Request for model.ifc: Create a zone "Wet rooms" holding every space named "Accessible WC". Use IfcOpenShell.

First a look at what the model holds.

```python
import ifcopenshell

model = ifcopenshell.open("model.ifc")
print(model.schema)
seen = {}
for space in model.by_type("IfcSpace"):
    seen[space.LongName] = seen.get(space.LongName, 0) + 1
for name, count in sorted(seen.items(), key=str):
    print(count, "x", name)
print("zones:", [z.Name for z in model.by_type("IfcZone")][:20])
```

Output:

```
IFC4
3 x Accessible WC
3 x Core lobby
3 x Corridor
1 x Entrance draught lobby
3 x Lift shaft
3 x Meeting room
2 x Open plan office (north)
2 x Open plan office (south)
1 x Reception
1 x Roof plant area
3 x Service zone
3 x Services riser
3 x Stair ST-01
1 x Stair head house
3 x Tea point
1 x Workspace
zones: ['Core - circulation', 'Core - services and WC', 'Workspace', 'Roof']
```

```python
import ifcopenshell
import ifcopenshell.api.group
import ifcopenshell.api.root

model = ifcopenshell.open("model.ifc")

names = {"Accessible WC"}
spaces = [s for s in model.by_type("IfcSpace") if s.LongName in names]

zone = ifcopenshell.api.root.create_entity(model, ifc_class="IfcZone", name="Wet rooms")
ifcopenshell.api.group.assign_group(model, products=spaces, group=zone)
print(len(spaces), "spaces in", zone.Name)

model.write("model_v2.ifc")
```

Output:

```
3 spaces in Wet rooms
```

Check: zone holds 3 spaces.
